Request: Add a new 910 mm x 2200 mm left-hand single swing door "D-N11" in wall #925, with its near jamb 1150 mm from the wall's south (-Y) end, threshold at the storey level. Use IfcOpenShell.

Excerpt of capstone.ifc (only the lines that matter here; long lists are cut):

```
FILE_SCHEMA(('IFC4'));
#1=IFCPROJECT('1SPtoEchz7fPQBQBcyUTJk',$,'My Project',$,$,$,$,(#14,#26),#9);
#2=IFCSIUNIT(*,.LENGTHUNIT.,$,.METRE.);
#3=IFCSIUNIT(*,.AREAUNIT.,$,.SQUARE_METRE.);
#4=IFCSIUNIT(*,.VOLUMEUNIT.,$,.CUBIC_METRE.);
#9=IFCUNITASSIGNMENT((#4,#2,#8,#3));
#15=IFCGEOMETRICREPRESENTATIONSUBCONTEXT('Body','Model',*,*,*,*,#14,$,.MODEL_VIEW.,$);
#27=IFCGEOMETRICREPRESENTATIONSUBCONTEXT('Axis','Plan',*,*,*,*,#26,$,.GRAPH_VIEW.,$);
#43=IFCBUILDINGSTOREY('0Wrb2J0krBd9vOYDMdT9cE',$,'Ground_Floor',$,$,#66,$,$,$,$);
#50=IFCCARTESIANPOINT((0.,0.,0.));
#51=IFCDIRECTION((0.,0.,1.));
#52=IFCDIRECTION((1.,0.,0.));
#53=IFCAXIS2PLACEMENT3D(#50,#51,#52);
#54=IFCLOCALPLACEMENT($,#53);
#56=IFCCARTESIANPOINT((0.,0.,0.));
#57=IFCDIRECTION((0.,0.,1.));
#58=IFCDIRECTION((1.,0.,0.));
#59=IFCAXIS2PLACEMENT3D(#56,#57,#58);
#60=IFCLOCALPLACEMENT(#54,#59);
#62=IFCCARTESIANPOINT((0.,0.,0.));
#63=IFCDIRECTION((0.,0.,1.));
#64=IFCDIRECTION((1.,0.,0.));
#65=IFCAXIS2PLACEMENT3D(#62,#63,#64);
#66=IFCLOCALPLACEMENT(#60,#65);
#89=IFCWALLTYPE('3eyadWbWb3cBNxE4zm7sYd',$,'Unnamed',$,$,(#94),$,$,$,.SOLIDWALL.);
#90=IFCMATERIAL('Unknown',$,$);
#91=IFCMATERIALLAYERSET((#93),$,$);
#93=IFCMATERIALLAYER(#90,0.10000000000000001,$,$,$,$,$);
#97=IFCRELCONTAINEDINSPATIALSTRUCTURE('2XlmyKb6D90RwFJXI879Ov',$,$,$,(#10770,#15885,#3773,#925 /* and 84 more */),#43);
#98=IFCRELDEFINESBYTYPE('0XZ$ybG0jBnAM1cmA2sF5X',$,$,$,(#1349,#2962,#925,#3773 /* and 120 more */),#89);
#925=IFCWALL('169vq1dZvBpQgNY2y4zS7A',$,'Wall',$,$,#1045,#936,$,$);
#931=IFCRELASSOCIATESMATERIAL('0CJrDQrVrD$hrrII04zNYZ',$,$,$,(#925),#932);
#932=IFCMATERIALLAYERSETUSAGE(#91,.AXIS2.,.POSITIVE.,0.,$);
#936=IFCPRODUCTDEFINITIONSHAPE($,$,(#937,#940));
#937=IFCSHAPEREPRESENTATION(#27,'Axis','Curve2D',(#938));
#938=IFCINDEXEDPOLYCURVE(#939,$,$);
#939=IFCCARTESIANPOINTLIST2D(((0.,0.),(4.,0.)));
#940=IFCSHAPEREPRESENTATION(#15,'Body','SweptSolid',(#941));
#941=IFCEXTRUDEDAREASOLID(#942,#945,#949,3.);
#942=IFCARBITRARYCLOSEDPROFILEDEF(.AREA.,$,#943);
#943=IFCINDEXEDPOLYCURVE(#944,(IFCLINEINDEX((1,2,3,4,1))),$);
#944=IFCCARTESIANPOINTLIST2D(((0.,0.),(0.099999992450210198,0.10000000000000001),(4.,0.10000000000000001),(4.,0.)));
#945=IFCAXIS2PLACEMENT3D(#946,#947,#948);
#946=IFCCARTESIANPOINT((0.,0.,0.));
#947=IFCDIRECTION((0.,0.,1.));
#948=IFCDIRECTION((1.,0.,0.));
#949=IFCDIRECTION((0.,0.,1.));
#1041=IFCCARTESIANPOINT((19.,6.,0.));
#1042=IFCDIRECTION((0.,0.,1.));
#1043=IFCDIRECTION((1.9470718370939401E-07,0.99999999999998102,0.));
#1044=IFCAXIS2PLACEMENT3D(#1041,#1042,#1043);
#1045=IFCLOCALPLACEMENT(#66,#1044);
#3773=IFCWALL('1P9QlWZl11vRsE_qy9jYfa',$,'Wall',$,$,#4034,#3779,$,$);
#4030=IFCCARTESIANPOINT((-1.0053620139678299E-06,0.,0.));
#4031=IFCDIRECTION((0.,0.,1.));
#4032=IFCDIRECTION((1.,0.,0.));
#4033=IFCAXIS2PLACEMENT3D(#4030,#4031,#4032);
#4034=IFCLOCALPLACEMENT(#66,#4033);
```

```python
import numpy as np
import ifcopenshell
import ifcopenshell.api.feature
import ifcopenshell.api.geometry
import ifcopenshell.api.root
import ifcopenshell.api.spatial
import ifcopenshell.geom
import ifcopenshell.util.element
import ifcopenshell.util.placement
import ifcopenshell.util.representation
import ifcopenshell.util.shape
import ifcopenshell.util.unit

model = ifcopenshell.open("capstone.ifc")
unit_scale = ifcopenshell.util.unit.calculate_unit_scale(model)
settings = ifcopenshell.geom.settings()


def volume(element):
    """Net volume in cubic metres, openings subtracted."""
    shape = ifcopenshell.geom.create_shape(settings, element)
    return ifcopenshell.util.shape.get_volume(shape.geometry)


wall = model.by_guid("169vq1dZvBpQgNY2y4zS7A")
storey = ifcopenshell.util.element.get_container(wall, ifc_class="IfcBuildingStorey")
context = ifcopenshell.util.representation.get_context(model, "Model", "Body", "MODEL_VIEW")
before = volume(wall)

width, height, from_end, sill = 0.91, 2.2, 1.15, 0.0  # metres

# The wall runs along its own X axis, and the end named is its -X end.
wall_shape = ifcopenshell.geom.create_shape(settings, wall)
x, y, z = ifcopenshell.util.shape.get_vertices(wall_shape.geometry).T
start = x.min() + from_end
face, thickness = float(y.min()), float(y.max() - y.min())
wall_matrix = ifcopenshell.util.placement.get_local_placement(wall.ObjectPlacement)
level = ifcopenshell.util.placement.get_local_placement(storey.ObjectPlacement)[2, 3]


def in_wall(x, y):
    """Placement at x, y metres in the wall's axes, at sill height."""
    matrix = wall_matrix.copy()
    matrix[:, 3] = wall_matrix @ np.array([x / unit_scale, y / unit_scale, 0.0, 1.0])
    matrix[2, 3] = level + sill / unit_scale
    return matrix


# Opening: a box that overshoots both wall faces by 50 mm.
opening = ifcopenshell.api.root.create_entity(model, ifc_class="IfcOpeningElement", predefined_type="OPENING")
box = ifcopenshell.api.geometry.add_wall_representation(
    model, context=context, length=width, height=height, thickness=thickness + 0.1
)
ifcopenshell.api.geometry.assign_representation(model, product=opening, representation=box)
ifcopenshell.api.geometry.edit_object_placement(model, product=opening, matrix=in_wall(start, face - 0.05), is_si=False)
ifcopenshell.api.feature.add_feature(model, feature=opening, element=wall)

door = ifcopenshell.api.root.create_entity(model, ifc_class="IfcDoor", name="D-N11", predefined_type="DOOR")
door.OverallWidth, door.OverallHeight = width / unit_scale, height / unit_scale
door.OperationType = "SINGLE_SWING_LEFT"
body = ifcopenshell.api.geometry.add_door_representation(
    model,
    context=context,
    overall_width=door.OverallWidth,
    overall_height=door.OverallHeight,
    operation_type="SINGLE_SWING_LEFT",
    lining_properties={"LiningDepth": thickness / unit_scale, "ThresholdDepth": thickness / unit_scale},
)
ifcopenshell.api.geometry.assign_representation(model, product=door, representation=body)
ifcopenshell.api.spatial.assign_container(model, products=[door], relating_structure=storey)
ifcopenshell.api.feature.add_filling(model, opening=opening, element=door)

# The lining spans the wall, so the door starts at the wall face.
ifcopenshell.api.geometry.edit_object_placement(model, product=door, matrix=in_wall(start, face), is_si=False)

after = volume(wall)

print(f"wall volume {before:.3f} -> {after:.3f} m3")

model.write("capstone_updated.ifc")
```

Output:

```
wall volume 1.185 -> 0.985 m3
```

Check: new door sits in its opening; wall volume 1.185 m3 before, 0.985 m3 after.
